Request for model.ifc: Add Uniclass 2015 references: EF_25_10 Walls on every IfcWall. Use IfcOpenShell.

First a look at what the model holds.

```python
import ifcopenshell

model = ifcopenshell.open("model.ifc")
print(model.schema)
print("classifications:", [c.Name for c in model.by_type("IfcClassification")])
for ifc_class in ("IfcDoor", "IfcRoof", "IfcStair", "IfcWall", "IfcWindow"):
    print(ifc_class, len(model.by_type(ifc_class)))
```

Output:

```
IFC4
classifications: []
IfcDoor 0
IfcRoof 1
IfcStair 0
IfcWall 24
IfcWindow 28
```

```python
import ifcopenshell
import ifcopenshell.api.classification

model = ifcopenshell.open("model.ifc")

system = ifcopenshell.api.classification.add_classification(model, classification="Uniclass 2015")

codes = {
    "IfcWall": ("EF_25_10", "Walls"),
}
for ifc_class, (code, name) in codes.items():
    products = model.by_type(ifc_class)
    ifcopenshell.api.classification.add_reference(
        model, products=products, classification=system, identification=code, name=name
    )
    print(code, len(products))

model.write("model-out.ifc")
```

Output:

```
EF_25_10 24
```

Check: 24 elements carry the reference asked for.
